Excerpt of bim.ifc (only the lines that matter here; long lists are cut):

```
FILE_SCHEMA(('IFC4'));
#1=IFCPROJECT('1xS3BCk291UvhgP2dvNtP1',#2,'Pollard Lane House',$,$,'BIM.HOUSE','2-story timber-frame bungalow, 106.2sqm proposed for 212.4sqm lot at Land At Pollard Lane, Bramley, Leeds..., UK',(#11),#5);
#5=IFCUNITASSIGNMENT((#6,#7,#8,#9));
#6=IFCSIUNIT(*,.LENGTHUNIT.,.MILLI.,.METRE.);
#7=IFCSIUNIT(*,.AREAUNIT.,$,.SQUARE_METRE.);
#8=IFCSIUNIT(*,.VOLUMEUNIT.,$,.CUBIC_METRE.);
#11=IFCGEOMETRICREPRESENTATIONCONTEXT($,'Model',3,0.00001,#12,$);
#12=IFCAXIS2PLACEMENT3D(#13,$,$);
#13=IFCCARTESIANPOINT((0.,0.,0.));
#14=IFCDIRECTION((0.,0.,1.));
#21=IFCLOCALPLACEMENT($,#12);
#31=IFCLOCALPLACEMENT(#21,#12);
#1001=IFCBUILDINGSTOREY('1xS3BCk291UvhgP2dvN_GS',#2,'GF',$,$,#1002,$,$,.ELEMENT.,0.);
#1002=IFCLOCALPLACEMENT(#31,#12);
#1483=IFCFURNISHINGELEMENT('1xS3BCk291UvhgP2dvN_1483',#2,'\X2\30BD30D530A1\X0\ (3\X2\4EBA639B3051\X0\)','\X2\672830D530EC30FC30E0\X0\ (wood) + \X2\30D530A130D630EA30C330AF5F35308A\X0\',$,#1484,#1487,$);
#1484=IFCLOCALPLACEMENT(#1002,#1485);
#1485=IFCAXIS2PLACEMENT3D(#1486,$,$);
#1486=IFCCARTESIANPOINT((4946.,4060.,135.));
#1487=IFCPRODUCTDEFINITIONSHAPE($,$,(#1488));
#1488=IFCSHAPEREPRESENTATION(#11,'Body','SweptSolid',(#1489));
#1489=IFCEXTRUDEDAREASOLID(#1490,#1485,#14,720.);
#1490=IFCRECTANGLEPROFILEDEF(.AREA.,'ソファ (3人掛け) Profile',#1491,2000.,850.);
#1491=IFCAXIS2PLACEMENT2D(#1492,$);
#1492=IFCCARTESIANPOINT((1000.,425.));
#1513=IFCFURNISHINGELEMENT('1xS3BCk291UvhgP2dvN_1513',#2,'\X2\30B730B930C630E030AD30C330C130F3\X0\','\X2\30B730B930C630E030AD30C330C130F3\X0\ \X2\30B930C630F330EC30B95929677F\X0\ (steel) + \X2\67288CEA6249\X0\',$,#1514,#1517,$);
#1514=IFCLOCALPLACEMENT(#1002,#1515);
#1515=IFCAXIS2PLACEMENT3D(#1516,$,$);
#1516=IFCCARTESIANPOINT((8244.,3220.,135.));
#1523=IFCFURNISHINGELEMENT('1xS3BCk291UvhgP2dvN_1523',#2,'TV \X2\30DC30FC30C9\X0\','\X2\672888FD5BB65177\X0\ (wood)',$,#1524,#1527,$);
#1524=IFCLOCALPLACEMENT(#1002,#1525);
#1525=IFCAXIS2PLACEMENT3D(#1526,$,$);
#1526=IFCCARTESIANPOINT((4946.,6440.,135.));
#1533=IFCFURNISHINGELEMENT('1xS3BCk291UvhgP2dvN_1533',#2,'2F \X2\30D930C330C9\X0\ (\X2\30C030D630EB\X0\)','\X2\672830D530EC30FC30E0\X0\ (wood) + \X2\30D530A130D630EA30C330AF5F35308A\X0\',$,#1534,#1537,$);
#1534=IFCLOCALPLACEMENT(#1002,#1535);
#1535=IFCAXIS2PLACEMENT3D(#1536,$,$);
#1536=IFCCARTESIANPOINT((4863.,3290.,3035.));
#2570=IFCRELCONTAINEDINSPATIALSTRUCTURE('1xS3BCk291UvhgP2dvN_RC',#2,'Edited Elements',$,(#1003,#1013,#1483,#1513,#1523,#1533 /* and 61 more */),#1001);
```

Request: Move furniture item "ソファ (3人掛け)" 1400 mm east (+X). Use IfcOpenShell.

```python
import ifcopenshell
import ifcopenshell.api.geometry
import ifcopenshell.util.placement

model = ifcopenshell.open("bim.ifc")

item = model.by_guid("1xS3BCk291UvhgP2dvN_1483")
matrix = ifcopenshell.util.placement.get_local_placement(item.ObjectPlacement)
matrix[0, 3] += 1400.0
ifcopenshell.api.geometry.edit_object_placement(model, product=item, matrix=matrix, is_si=False)

print(ifcopenshell.util.placement.get_local_placement(item.ObjectPlacement).round(3) + 0.0)

model.write("bim_updated.ifc")
```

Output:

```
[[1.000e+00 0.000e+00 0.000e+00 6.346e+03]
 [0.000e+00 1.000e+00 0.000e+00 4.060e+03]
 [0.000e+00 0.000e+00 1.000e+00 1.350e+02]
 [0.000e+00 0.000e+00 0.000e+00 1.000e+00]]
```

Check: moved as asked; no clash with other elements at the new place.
